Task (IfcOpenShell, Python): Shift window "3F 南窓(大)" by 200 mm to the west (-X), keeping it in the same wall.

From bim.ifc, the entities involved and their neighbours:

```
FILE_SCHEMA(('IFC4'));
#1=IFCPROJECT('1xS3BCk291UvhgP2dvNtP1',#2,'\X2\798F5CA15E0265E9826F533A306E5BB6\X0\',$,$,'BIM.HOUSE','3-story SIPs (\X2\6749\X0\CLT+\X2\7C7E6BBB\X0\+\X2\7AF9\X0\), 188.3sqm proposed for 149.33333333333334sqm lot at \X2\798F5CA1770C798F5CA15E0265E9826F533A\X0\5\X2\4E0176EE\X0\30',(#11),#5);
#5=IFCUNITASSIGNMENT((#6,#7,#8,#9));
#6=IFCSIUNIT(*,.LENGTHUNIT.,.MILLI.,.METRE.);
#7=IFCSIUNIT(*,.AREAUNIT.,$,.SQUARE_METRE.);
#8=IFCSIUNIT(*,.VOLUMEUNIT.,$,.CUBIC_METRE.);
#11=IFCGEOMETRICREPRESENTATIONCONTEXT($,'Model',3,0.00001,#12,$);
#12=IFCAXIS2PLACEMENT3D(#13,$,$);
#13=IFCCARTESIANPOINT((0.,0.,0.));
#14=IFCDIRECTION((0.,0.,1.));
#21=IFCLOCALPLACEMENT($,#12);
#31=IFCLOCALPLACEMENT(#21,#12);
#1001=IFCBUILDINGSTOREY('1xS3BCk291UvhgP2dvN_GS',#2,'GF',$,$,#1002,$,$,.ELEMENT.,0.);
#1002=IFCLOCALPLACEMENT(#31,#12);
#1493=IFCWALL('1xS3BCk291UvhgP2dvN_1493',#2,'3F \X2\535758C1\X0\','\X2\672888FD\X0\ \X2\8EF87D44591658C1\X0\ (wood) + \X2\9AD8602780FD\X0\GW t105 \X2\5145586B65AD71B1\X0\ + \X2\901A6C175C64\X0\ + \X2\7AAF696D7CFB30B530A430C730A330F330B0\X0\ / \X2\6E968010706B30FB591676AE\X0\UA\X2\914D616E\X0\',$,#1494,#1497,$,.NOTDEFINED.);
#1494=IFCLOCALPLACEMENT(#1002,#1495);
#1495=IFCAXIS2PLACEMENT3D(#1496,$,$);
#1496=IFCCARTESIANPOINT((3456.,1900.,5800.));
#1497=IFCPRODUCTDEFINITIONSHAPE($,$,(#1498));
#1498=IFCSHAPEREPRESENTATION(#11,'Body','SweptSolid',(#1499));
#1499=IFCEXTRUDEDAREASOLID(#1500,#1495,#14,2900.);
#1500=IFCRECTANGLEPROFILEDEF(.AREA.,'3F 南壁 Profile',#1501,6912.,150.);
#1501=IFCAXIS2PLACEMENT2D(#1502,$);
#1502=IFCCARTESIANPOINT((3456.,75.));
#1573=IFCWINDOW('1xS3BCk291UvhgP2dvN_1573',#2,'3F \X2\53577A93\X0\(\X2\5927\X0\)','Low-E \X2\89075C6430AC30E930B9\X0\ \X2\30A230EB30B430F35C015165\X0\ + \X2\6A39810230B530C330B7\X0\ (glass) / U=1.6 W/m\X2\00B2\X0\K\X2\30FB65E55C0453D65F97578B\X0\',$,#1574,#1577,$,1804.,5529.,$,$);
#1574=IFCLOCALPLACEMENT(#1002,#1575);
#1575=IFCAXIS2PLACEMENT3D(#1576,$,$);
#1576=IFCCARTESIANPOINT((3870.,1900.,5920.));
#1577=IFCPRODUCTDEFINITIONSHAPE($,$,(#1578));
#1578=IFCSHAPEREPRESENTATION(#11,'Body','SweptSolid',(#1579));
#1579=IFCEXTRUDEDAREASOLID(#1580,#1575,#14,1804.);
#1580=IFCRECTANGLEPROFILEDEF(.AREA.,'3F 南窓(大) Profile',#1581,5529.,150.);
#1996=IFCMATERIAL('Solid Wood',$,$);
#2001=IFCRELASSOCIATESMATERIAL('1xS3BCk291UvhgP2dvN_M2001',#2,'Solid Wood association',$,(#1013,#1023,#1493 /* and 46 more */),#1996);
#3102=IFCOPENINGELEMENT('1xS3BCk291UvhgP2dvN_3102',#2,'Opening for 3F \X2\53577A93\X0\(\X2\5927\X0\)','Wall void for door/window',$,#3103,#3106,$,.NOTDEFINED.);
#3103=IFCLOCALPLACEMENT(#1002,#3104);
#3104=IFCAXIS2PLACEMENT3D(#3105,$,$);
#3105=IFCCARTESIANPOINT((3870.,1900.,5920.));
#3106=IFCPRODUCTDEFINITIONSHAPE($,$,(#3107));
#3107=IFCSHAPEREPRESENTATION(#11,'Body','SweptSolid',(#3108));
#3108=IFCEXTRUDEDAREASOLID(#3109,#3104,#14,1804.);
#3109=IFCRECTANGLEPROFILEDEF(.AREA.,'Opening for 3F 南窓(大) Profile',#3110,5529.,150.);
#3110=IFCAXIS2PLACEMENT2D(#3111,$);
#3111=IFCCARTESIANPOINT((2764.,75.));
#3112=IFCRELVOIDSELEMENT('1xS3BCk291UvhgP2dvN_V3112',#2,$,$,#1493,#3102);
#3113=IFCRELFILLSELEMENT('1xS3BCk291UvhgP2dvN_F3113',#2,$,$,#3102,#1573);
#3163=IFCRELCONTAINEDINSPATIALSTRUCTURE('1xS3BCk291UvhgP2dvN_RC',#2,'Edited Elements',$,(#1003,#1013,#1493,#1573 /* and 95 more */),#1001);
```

```python
import ifcopenshell
import ifcopenshell.api.geometry
import ifcopenshell.util.placement

model = ifcopenshell.open("bim.ifc")

window = model.by_id(1573)
opening = window.FillsVoids[0].RelatingOpeningElement
wall = opening.VoidsElements[0].RelatingBuildingElement

wall_matrix = ifcopenshell.util.placement.get_local_placement(wall.ObjectPlacement)
shift = wall_matrix[:3, 0] * -200.0
before = ifcopenshell.util.placement.get_local_placement(window.ObjectPlacement)[:3, 3].copy()

# The window is not placed relative to its opening, so move both.
for product in (opening, window):
    matrix = ifcopenshell.util.placement.get_local_placement(product.ObjectPlacement)
    matrix[:3, 3] += shift
    ifcopenshell.api.geometry.edit_object_placement(model, product=product, matrix=matrix, is_si=False)

after = ifcopenshell.util.placement.get_local_placement(window.ObjectPlacement)[:3, 3]
print("window moved by", (after - before).round(3) + 0.0)

model.write("bim_rev.ifc")
```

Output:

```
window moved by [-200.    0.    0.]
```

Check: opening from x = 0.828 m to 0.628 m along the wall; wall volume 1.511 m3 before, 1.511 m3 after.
